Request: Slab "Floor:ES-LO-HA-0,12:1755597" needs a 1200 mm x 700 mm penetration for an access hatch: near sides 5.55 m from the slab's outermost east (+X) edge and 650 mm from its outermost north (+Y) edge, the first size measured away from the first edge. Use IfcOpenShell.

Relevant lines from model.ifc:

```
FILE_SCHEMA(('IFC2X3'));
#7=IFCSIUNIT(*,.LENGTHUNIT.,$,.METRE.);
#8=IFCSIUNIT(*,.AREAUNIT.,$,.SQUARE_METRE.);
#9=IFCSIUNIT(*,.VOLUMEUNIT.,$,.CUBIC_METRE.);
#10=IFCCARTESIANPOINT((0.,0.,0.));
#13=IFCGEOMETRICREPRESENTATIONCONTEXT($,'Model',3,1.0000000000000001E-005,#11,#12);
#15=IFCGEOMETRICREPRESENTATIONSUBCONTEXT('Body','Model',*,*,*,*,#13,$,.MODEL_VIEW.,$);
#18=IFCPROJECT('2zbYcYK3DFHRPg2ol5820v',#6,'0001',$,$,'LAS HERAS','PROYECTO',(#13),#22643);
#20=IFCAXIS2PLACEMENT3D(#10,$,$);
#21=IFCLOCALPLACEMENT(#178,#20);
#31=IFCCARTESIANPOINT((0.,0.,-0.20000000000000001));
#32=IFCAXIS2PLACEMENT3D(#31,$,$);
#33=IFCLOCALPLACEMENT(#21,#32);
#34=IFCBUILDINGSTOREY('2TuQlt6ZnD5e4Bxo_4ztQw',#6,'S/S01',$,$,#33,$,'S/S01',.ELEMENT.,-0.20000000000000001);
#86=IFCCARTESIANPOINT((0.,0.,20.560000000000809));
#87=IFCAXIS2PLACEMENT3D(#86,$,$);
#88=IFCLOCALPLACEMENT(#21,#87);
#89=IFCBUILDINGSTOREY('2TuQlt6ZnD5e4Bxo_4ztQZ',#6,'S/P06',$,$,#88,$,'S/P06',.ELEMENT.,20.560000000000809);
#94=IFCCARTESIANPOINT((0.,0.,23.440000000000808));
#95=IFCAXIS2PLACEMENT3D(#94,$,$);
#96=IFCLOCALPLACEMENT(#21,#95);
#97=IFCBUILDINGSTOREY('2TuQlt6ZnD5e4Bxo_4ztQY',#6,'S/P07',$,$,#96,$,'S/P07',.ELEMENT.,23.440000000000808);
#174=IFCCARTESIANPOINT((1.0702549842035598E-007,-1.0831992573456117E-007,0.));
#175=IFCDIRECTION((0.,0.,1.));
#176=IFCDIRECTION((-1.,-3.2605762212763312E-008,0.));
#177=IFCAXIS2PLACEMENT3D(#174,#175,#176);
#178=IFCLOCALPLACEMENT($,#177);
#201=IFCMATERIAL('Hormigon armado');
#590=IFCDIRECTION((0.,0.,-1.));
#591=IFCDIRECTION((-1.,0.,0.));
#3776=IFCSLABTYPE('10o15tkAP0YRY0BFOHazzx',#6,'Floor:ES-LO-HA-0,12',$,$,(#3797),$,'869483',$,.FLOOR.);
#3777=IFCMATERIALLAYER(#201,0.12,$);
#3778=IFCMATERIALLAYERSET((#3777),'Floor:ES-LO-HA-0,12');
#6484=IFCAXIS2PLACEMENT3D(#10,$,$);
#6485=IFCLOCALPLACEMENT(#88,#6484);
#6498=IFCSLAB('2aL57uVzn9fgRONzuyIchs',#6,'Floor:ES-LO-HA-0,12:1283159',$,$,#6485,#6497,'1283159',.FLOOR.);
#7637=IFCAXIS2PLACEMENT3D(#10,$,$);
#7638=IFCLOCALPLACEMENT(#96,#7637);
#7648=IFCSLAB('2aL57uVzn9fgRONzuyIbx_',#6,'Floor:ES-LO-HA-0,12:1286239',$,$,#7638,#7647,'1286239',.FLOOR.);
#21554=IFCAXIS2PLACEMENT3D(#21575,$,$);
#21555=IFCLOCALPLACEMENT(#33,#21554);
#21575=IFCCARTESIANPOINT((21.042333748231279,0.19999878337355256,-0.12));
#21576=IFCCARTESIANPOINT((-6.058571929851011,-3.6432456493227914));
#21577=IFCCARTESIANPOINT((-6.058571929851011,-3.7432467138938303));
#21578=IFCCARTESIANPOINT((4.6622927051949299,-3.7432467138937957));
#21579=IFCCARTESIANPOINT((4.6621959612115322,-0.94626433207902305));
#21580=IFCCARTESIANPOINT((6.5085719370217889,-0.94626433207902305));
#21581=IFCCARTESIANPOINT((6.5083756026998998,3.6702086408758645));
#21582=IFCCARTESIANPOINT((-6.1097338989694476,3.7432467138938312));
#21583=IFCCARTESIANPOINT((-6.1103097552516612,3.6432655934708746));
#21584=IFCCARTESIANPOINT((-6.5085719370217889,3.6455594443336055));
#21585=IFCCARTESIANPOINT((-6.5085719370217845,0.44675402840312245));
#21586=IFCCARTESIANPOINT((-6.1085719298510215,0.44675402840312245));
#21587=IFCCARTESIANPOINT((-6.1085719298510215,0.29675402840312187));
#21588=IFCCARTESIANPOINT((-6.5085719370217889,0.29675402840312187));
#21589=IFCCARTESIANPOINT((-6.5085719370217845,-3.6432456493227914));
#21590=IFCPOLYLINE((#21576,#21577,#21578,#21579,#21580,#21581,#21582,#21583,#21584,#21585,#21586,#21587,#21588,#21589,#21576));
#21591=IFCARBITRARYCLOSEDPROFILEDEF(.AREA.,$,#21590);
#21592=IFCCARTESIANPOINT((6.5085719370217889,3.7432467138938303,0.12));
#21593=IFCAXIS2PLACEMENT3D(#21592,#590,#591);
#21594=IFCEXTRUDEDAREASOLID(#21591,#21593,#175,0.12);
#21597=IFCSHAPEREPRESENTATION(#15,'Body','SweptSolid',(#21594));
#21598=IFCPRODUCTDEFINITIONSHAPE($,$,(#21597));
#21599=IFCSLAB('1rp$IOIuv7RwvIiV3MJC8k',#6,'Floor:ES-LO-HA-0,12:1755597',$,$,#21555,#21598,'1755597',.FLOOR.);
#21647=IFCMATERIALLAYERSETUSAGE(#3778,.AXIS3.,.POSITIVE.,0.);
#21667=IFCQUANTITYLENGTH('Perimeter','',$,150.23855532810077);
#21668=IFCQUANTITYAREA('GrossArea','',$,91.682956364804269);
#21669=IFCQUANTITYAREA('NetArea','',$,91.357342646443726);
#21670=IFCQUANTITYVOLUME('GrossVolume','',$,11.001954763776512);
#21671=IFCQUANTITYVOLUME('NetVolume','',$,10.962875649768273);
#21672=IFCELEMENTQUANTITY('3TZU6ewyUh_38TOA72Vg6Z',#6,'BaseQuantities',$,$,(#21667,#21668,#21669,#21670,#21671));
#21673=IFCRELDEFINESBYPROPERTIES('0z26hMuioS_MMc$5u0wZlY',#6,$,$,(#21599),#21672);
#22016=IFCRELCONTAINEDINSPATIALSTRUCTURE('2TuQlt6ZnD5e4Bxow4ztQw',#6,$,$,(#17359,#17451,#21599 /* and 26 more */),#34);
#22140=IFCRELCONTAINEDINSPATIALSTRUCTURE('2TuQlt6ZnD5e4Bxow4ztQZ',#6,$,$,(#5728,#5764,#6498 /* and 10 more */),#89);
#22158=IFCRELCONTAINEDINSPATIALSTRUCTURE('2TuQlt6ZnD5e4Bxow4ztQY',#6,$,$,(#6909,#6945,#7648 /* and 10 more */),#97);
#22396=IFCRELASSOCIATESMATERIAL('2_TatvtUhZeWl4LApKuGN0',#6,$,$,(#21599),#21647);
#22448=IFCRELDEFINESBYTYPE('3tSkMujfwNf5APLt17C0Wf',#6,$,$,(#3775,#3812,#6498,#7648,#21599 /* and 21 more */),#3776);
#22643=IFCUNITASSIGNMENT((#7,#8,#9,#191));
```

```python
import numpy as np
import ifcopenshell
import ifcopenshell.api.feature
import ifcopenshell.api.geometry
import ifcopenshell.api.pset
import ifcopenshell.api.root
import ifcopenshell.geom
import ifcopenshell.util.element
import ifcopenshell.util.placement
import ifcopenshell.util.representation
import ifcopenshell.util.shape
import ifcopenshell.util.unit

model = ifcopenshell.open("model.ifc")
unit_scale = ifcopenshell.util.unit.calculate_unit_scale(model)
area_scale = ifcopenshell.util.unit.calculate_unit_scale(model, "AREAUNIT")
volume_scale = ifcopenshell.util.unit.calculate_unit_scale(model, "VOLUMEUNIT")
settings = ifcopenshell.geom.settings()


def volume(element):
    """Net volume in cubic metres, openings subtracted."""
    shape = ifcopenshell.geom.create_shape(settings, element)
    return ifcopenshell.util.shape.get_volume(shape.geometry)


slab = model.by_guid("1rp$IOIuv7RwvIiV3MJC8k")
before = volume(slab)

# Extent in the slab's own axes, in metres. The edges named are its -X and -Y sides.
slab_shape = ifcopenshell.geom.create_shape(settings, slab)
vertices = ifcopenshell.util.shape.get_vertices(slab_shape.geometry)
x_min, y_min, bottom = vertices.min(axis=0)
top = vertices[:, 2].max()

opening = ifcopenshell.api.root.create_entity(model, ifc_class="IfcOpeningElement", name="Access hatch opening")
context = ifcopenshell.util.representation.get_context(model, "Model", "Body", "MODEL_VIEW")
width, depth = 1.2, 0.7
outline = [(0.0, 0.0), (width, 0.0), (width, depth), (0.0, depth), (0.0, 0.0)]
# Overshoot both faces by 50 mm so the cut is clean.
shape = ifcopenshell.api.geometry.add_slab_representation(
    model, context=context, depth=top - bottom + 0.1, polyline=outline
)
ifcopenshell.api.geometry.assign_representation(model, product=opening, representation=shape)

matrix = ifcopenshell.util.placement.get_local_placement(slab.ObjectPlacement)
matrix[:, 3] = matrix @ np.append(np.array([x_min + 5.55, y_min + 0.65, bottom - 0.05]) / unit_scale, 1.0)
ifcopenshell.api.geometry.edit_object_placement(model, product=opening, matrix=matrix, is_si=False)
ifcopenshell.api.feature.add_feature(model, feature=opening, element=slab)

after = volume(slab)

# Update the slab's stored quantities.
qto = model.by_id(ifcopenshell.util.element.get_pset(slab, "BaseQuantities", should_inherit=False)["id"])
ifcopenshell.api.pset.edit_qto(model, qto=qto, properties={
    "NetArea": after / (top - bottom) / area_scale,
    "NetVolume": after / volume_scale,
})

print(f"slab volume {before:.3f} -> {after:.3f} m3")

model.write("model_edited.ifc")
```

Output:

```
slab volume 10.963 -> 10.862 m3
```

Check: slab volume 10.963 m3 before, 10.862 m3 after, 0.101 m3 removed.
